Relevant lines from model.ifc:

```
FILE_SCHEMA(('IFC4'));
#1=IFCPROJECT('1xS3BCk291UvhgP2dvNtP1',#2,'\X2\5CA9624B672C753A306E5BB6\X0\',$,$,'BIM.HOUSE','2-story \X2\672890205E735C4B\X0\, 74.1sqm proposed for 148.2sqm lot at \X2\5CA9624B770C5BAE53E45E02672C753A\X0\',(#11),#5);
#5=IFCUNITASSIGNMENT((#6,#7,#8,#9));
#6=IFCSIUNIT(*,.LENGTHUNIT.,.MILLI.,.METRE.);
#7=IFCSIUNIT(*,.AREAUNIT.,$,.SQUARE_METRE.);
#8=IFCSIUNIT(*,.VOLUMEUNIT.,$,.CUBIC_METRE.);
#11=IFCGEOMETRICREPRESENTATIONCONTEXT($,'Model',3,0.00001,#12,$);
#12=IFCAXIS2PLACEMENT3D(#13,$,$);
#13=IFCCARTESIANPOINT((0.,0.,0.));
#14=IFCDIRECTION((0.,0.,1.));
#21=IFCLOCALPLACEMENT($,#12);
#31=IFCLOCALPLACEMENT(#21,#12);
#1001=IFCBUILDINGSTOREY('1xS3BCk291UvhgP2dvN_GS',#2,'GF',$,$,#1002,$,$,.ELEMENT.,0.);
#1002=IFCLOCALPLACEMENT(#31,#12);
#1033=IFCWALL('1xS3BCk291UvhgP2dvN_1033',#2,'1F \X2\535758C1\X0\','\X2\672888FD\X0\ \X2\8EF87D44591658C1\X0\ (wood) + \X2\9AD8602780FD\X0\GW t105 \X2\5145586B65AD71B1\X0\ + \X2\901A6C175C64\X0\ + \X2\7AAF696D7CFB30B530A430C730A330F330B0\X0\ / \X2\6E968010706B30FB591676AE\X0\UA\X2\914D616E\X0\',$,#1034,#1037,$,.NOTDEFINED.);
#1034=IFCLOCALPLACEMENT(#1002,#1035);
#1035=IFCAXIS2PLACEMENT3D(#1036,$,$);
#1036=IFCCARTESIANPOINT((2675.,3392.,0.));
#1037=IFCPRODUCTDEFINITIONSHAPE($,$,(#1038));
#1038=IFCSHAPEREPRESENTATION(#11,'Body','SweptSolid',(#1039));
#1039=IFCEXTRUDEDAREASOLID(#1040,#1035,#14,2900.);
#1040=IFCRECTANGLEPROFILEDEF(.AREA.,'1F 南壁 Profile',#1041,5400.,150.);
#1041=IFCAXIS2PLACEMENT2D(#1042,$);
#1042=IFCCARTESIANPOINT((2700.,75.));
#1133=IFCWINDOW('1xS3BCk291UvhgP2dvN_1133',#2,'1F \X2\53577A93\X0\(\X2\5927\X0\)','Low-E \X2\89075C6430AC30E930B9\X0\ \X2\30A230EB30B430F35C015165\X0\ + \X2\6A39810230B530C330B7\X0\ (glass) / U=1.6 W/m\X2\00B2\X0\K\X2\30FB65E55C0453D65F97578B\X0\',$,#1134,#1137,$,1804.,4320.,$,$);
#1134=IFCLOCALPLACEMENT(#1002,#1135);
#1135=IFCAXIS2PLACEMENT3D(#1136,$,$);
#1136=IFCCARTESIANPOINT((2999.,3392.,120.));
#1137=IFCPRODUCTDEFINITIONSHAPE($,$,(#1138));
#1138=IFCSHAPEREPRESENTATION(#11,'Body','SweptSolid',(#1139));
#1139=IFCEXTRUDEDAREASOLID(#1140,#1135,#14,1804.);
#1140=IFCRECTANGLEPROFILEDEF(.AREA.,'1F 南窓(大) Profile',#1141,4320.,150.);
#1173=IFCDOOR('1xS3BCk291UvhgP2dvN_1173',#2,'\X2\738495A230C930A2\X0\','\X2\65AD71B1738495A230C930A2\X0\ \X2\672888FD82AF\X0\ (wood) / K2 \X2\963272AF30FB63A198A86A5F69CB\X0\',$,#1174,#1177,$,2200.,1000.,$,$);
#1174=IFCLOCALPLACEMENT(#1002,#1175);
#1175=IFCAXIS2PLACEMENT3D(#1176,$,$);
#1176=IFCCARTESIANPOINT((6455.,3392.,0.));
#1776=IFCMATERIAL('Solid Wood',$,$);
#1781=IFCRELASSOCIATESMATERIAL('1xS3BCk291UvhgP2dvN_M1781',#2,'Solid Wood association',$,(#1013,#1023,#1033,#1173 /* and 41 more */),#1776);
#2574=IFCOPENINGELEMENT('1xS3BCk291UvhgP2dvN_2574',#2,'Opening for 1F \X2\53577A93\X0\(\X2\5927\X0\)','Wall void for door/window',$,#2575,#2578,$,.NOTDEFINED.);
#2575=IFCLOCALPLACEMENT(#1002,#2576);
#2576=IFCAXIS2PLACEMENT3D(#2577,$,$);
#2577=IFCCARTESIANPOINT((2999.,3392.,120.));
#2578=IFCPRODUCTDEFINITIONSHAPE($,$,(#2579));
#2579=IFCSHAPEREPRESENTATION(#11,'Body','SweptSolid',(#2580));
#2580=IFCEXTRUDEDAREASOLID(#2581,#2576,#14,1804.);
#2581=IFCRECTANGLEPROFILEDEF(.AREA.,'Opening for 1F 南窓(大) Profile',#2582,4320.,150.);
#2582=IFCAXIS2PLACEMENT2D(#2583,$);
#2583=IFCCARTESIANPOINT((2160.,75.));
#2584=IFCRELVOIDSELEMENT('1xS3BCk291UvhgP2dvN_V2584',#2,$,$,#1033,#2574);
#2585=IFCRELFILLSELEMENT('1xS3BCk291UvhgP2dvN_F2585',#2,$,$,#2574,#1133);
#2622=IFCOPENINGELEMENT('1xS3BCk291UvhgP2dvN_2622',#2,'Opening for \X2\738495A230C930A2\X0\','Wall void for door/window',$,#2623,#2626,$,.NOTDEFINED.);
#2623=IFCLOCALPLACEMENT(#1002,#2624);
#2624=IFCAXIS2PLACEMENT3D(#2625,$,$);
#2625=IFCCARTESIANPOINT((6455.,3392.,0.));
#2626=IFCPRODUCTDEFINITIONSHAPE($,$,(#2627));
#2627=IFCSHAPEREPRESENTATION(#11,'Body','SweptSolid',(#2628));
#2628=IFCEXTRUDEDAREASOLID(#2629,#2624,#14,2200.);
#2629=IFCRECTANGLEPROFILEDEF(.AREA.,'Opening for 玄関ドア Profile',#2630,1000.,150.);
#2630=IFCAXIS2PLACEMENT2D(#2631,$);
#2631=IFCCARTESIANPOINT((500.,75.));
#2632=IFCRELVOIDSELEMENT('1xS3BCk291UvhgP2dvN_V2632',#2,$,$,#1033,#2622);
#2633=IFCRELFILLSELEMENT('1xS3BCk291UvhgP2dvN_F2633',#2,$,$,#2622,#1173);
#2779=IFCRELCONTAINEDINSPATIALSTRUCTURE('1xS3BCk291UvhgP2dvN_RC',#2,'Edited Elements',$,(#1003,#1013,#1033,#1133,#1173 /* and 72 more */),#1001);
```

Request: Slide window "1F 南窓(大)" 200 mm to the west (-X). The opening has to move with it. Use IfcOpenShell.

```python
import ifcopenshell
import ifcopenshell.api.geometry
import ifcopenshell.util.placement
import ifcopenshell.util.unit

model = ifcopenshell.open("model.ifc")
unit_scale = ifcopenshell.util.unit.calculate_unit_scale(model)

window = model.by_id(1133)
opening = window.FillsVoids[0].RelatingOpeningElement
wall = opening.VoidsElements[0].RelatingBuildingElement

wall_matrix = ifcopenshell.util.placement.get_local_placement(wall.ObjectPlacement)
shift = wall_matrix[:3, 0] * -0.2 / unit_scale
before = ifcopenshell.util.placement.get_local_placement(window.ObjectPlacement)[:3, 3].copy()

# The window is not placed relative to its opening, so move both.
for product in (opening, window):
    matrix = ifcopenshell.util.placement.get_local_placement(product.ObjectPlacement)
    matrix[:3, 3] += shift
    ifcopenshell.api.geometry.edit_object_placement(model, product=product, matrix=matrix, is_si=False)

after = ifcopenshell.util.placement.get_local_placement(window.ObjectPlacement)[:3, 3]
print("window moved by", (after - before).round(3) + 0.0)

model.write("model-out.ifc")
```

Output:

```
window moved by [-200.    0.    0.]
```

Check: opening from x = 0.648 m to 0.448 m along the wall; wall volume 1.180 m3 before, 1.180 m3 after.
